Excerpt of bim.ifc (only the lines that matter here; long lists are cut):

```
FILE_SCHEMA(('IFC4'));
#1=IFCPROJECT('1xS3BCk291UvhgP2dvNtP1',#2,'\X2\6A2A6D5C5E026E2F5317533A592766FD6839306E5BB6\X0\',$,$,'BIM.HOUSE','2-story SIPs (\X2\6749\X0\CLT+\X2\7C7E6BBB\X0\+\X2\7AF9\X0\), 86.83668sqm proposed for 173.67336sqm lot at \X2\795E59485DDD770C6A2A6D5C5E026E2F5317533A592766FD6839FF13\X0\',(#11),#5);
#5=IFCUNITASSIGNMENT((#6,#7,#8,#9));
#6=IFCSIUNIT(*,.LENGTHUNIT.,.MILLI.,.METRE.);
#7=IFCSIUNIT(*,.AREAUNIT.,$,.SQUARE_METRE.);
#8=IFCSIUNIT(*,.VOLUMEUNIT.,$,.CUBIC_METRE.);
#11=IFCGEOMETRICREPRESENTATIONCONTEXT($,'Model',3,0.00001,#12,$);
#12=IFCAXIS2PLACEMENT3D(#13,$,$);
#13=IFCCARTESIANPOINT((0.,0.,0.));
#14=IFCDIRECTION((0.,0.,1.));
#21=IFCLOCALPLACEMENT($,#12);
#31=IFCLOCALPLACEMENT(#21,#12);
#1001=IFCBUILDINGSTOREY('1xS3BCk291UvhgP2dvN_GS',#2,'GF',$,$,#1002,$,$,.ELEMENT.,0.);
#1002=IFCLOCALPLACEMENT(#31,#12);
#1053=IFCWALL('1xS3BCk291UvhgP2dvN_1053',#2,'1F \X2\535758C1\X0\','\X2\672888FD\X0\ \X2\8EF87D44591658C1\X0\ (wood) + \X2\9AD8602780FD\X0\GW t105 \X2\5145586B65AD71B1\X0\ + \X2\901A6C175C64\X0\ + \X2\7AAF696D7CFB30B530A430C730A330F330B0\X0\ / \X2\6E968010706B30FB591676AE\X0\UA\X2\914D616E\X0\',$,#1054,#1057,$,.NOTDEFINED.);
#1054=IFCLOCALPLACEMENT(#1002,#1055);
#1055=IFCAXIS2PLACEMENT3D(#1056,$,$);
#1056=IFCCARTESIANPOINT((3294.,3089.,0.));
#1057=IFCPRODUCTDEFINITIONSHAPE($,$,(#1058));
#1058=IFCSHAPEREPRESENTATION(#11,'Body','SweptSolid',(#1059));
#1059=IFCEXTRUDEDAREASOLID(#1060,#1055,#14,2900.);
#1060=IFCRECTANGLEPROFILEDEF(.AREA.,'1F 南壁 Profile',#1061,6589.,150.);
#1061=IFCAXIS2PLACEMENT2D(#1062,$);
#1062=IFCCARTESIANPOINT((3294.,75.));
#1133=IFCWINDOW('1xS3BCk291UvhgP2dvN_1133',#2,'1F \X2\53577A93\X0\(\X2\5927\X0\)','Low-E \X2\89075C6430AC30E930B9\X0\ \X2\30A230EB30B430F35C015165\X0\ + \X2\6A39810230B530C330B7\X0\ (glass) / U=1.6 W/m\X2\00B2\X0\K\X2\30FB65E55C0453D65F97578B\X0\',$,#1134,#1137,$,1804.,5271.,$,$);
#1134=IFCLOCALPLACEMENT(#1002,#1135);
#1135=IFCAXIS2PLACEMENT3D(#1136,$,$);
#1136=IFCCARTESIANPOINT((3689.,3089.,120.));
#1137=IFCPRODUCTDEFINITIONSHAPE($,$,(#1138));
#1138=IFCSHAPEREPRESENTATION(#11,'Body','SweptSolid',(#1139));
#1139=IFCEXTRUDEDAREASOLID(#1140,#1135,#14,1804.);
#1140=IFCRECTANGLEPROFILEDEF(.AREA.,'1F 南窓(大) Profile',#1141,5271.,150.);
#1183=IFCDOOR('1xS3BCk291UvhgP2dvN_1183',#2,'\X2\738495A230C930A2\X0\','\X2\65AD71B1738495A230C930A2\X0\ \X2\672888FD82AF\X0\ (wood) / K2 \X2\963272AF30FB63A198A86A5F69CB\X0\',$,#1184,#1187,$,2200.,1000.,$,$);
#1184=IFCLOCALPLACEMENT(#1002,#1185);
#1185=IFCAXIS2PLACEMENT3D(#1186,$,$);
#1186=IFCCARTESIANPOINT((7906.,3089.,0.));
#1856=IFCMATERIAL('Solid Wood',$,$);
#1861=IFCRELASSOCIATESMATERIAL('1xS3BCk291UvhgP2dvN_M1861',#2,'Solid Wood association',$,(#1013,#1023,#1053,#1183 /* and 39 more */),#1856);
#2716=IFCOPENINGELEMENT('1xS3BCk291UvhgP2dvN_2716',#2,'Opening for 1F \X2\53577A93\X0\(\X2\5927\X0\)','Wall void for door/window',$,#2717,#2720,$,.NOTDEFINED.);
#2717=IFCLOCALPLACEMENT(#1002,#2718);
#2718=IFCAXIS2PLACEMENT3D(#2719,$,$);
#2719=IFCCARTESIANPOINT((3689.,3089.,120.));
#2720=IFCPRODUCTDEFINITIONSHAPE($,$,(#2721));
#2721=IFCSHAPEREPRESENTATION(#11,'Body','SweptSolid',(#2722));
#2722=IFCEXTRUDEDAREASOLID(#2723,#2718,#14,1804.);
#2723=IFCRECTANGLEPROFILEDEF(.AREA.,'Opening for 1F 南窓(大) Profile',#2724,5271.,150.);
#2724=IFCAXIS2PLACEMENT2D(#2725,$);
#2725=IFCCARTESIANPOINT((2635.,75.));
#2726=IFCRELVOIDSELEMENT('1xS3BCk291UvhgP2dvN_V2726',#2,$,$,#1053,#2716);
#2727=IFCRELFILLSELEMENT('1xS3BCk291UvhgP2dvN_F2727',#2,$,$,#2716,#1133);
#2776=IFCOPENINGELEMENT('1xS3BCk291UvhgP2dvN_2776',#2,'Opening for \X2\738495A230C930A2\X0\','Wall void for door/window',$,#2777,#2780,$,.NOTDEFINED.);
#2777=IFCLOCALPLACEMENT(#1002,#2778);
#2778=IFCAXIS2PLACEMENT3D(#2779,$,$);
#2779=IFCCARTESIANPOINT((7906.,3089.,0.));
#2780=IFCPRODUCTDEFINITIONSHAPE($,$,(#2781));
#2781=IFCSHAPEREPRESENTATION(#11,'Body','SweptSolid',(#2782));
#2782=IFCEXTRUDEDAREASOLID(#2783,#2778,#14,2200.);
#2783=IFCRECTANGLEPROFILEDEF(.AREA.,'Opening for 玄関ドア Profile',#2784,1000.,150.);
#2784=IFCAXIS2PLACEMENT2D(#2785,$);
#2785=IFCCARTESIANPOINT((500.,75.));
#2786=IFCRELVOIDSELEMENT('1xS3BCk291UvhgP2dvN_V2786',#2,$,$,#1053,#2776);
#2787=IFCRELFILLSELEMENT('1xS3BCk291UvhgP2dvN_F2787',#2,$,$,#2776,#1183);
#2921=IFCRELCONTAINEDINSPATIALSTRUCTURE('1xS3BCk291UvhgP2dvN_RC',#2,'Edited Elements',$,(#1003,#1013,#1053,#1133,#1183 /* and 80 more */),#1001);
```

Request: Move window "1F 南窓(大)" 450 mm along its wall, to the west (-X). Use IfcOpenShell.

```python
import ifcopenshell
import ifcopenshell.api.geometry
import ifcopenshell.util.placement

model = ifcopenshell.open("bim.ifc")

window = model.by_guid("1xS3BCk291UvhgP2dvN_1133")
opening = window.FillsVoids[0].RelatingOpeningElement
wall = opening.VoidsElements[0].RelatingBuildingElement

wall_matrix = ifcopenshell.util.placement.get_local_placement(wall.ObjectPlacement)
shift = wall_matrix[:3, 0] * -450.0
before = ifcopenshell.util.placement.get_local_placement(window.ObjectPlacement)[:3, 3].copy()

# The window is not placed relative to its opening, so move both.
for product in (opening, window):
    matrix = ifcopenshell.util.placement.get_local_placement(product.ObjectPlacement)
    matrix[:3, 3] += shift
    ifcopenshell.api.geometry.edit_object_placement(model, product=product, matrix=matrix, is_si=False)

after = ifcopenshell.util.placement.get_local_placement(window.ObjectPlacement)[:3, 3]
print("window moved by", (after - before).round(3) + 0.0)

model.write("bim_v2.ifc")
```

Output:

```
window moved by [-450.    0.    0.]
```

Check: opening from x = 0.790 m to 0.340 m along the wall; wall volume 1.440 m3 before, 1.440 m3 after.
